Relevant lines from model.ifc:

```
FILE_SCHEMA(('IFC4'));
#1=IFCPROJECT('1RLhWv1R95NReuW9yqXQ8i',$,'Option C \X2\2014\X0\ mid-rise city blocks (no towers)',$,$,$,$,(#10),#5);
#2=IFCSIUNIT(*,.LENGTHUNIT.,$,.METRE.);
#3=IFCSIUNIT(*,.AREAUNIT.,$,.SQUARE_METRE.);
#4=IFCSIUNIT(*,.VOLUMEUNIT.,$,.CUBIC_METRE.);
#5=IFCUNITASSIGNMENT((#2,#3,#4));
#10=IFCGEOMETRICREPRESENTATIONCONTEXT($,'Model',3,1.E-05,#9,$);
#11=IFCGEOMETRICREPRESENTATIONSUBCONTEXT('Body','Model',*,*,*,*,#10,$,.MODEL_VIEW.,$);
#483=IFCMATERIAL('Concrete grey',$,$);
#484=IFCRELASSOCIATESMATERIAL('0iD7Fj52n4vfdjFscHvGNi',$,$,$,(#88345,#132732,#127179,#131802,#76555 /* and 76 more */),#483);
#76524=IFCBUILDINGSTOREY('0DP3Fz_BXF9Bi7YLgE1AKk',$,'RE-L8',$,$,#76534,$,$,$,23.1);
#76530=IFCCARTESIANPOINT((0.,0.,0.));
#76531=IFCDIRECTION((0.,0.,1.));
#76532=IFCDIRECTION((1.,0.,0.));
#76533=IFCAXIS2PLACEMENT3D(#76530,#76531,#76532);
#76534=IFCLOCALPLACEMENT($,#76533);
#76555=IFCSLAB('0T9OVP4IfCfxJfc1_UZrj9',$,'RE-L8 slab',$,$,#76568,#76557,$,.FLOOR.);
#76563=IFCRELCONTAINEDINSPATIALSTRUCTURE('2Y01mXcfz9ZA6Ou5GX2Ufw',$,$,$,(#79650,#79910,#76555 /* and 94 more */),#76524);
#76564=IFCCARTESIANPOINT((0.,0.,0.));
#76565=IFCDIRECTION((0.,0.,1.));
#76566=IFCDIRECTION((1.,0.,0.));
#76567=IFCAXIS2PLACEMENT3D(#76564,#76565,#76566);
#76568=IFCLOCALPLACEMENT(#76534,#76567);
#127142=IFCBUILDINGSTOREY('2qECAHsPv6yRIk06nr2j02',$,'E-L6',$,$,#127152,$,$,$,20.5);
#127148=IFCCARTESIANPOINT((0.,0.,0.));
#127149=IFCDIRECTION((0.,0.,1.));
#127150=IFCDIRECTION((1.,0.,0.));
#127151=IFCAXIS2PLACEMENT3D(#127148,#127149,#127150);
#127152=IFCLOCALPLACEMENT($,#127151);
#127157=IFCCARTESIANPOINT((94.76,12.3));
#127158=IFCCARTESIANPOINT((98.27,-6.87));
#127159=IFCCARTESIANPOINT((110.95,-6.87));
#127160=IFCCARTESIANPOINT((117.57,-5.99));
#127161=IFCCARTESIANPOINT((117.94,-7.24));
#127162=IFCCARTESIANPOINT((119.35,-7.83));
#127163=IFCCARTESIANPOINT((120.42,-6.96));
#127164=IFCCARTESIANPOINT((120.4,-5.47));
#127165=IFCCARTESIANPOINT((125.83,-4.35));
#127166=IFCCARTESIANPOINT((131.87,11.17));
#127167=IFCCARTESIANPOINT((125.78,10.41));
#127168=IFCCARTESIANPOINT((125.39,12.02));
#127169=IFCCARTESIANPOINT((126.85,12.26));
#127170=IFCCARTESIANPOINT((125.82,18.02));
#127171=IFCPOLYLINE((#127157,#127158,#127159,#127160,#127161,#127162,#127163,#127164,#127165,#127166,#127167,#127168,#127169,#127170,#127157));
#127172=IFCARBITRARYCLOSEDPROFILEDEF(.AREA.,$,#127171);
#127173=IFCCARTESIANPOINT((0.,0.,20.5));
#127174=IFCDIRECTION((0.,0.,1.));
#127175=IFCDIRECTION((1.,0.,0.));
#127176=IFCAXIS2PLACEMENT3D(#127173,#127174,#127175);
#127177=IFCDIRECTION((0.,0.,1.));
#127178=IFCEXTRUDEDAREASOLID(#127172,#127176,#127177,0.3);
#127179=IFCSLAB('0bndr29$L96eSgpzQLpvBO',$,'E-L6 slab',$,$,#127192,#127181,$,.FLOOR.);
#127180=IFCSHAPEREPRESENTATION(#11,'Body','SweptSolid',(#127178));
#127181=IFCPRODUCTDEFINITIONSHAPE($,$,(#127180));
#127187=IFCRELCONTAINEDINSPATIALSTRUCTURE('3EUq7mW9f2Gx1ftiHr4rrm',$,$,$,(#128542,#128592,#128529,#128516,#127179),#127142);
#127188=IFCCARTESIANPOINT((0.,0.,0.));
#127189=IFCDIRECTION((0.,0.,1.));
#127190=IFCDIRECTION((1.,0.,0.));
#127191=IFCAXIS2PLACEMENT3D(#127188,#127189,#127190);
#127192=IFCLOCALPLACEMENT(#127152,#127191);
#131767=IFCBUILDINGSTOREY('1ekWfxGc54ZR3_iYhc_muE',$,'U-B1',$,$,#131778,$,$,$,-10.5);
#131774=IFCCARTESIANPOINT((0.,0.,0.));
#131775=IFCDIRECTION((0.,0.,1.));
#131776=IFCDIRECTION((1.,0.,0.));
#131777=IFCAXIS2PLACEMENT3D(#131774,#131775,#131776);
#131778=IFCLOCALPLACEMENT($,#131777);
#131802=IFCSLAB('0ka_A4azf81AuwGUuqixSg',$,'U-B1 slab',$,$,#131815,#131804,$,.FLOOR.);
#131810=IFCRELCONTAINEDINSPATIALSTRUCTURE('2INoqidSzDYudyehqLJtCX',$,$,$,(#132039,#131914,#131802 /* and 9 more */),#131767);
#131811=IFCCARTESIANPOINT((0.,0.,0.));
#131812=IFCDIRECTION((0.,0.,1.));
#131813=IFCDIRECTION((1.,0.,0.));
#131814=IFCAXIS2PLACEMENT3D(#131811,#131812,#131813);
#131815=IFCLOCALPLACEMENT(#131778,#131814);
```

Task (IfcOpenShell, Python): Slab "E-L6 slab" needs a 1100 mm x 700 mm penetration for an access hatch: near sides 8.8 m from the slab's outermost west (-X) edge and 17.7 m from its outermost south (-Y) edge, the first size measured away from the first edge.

```python
import numpy as np
import ifcopenshell
import ifcopenshell.api.feature
import ifcopenshell.api.geometry
import ifcopenshell.api.root
import ifcopenshell.geom
import ifcopenshell.util.placement
import ifcopenshell.util.representation
import ifcopenshell.util.shape
import ifcopenshell.util.unit

model = ifcopenshell.open("model.ifc")
unit_scale = ifcopenshell.util.unit.calculate_unit_scale(model)
settings = ifcopenshell.geom.settings()


def volume(element):
    """Net volume in cubic metres, openings subtracted."""
    shape = ifcopenshell.geom.create_shape(settings, element)
    return ifcopenshell.util.shape.get_volume(shape.geometry)


slab = model.by_id(127179)
before = volume(slab)

# Extent in the slab's own axes, in metres. The edges named are its -X and -Y sides.
slab_shape = ifcopenshell.geom.create_shape(settings, slab)
vertices = ifcopenshell.util.shape.get_vertices(slab_shape.geometry)
x_min, y_min, bottom = vertices.min(axis=0)
top = vertices[:, 2].max()

opening = ifcopenshell.api.root.create_entity(model, ifc_class="IfcOpeningElement", name="Access hatch opening", predefined_type="OPENING")
context = ifcopenshell.util.representation.get_context(model, "Model", "Body", "MODEL_VIEW")
width, depth = 1.1, 0.7
outline = [(0.0, 0.0), (width, 0.0), (width, depth), (0.0, depth), (0.0, 0.0)]
# Overshoot both faces by 50 mm so the cut is clean.
shape = ifcopenshell.api.geometry.add_slab_representation(
    model, context=context, depth=top - bottom + 0.1, polyline=outline
)
ifcopenshell.api.geometry.assign_representation(model, product=opening, representation=shape)

matrix = ifcopenshell.util.placement.get_local_placement(slab.ObjectPlacement)
matrix[:, 3] = matrix @ np.append(np.array([x_min + 8.8, y_min + 17.7, bottom - 0.05]) / unit_scale, 1.0)
ifcopenshell.api.geometry.edit_object_placement(model, product=opening, matrix=matrix, is_si=False)
ifcopenshell.api.feature.add_feature(model, feature=opening, element=slab)

after = volume(slab)

print(f"slab volume {before:.3f} -> {after:.3f} m3")

model.write("model_v2.ifc")
```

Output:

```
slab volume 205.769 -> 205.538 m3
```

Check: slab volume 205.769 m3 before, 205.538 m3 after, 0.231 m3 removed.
